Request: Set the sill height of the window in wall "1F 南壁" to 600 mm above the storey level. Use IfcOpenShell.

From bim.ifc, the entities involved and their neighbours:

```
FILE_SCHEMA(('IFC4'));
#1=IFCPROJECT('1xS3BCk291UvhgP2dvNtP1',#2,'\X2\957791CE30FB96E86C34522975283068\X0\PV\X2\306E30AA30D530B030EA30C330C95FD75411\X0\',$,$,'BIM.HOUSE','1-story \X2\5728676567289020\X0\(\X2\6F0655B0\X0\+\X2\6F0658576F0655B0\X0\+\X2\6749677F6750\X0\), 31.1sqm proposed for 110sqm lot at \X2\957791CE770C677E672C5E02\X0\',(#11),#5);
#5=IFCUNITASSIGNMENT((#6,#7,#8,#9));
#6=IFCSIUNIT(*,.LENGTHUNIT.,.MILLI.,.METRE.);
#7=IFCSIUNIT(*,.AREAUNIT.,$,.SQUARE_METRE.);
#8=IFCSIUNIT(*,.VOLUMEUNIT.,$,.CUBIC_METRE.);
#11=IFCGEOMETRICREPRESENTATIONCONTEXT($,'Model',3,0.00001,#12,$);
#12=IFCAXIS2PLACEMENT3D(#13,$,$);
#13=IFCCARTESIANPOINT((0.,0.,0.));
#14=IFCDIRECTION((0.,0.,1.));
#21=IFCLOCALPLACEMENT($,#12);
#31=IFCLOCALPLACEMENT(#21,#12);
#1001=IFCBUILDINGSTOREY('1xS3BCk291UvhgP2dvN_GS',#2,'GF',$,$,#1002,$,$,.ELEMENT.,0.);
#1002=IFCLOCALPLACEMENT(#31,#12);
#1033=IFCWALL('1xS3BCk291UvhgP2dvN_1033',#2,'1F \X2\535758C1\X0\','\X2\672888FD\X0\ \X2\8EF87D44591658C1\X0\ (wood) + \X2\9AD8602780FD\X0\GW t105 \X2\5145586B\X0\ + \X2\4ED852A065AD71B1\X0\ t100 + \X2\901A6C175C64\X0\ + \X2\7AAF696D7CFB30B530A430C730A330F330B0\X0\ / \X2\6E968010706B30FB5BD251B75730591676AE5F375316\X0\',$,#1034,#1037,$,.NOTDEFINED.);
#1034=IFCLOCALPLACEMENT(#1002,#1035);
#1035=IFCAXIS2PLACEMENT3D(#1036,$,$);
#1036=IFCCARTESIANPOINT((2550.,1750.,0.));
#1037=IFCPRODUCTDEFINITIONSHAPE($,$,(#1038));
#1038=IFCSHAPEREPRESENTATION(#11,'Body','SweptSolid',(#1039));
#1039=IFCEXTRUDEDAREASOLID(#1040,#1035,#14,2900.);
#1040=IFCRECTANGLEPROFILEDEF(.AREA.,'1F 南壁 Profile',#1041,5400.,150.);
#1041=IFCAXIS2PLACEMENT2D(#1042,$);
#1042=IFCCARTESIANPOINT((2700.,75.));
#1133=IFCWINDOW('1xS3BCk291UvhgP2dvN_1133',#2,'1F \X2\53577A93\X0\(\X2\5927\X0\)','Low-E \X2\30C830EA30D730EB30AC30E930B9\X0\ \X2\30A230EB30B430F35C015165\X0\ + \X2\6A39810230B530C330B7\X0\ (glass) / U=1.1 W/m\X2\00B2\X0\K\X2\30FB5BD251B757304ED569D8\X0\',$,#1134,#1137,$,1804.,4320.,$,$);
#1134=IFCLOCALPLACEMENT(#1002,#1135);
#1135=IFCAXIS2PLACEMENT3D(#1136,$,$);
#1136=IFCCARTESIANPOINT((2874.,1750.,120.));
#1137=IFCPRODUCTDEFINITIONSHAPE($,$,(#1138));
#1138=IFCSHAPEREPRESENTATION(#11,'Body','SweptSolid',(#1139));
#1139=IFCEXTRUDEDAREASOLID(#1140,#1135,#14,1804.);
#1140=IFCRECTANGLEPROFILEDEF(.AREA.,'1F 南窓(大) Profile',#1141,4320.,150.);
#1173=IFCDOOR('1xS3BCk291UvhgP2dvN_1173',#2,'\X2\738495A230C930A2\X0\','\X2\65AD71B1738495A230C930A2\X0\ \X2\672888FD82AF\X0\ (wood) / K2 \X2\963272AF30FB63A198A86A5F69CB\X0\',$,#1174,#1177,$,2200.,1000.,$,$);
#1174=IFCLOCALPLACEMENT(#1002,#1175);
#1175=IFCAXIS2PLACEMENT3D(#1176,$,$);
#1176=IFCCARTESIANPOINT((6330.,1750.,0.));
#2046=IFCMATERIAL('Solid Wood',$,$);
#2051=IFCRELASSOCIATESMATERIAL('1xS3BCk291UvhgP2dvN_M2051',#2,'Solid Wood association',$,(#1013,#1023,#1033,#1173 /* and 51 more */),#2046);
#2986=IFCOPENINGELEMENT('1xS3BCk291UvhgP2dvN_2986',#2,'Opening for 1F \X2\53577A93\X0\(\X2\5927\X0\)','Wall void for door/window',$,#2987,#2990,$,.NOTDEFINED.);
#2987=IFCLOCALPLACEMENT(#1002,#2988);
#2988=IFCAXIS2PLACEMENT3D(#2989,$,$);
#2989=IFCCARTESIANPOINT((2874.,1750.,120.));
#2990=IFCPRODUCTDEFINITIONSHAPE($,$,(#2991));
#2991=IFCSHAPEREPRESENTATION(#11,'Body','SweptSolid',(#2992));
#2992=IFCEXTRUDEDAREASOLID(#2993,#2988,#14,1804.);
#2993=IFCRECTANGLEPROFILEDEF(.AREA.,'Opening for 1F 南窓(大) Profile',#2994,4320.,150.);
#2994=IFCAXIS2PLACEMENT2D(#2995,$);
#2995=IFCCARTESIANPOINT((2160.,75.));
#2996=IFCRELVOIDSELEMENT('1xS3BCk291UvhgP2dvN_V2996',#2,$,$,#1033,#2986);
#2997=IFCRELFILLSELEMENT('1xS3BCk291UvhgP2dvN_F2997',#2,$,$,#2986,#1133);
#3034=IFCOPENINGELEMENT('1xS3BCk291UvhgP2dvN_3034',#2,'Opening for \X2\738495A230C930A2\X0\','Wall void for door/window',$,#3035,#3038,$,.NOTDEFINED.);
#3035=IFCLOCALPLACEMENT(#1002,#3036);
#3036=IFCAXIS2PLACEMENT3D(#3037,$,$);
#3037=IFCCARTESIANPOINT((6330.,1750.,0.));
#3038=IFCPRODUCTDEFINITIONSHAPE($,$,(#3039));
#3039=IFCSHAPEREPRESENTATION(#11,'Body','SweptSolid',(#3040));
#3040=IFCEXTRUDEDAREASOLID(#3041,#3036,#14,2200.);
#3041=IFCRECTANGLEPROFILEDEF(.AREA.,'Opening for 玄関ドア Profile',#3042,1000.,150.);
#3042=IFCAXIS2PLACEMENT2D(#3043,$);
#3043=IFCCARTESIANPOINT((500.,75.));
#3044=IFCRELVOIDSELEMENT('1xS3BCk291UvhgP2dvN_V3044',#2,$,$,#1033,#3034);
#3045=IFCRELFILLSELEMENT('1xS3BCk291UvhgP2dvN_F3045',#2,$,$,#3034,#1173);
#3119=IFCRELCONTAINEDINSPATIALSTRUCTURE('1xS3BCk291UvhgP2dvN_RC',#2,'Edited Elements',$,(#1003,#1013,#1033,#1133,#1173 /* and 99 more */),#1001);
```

```python
import numpy as np
import ifcopenshell
import ifcopenshell.api.geometry
import ifcopenshell.geom
import ifcopenshell.util.element
import ifcopenshell.util.placement
import ifcopenshell.util.shape
import ifcopenshell.util.unit

model = ifcopenshell.open("bim.ifc")
unit_scale = ifcopenshell.util.unit.calculate_unit_scale(model)

window = model.by_guid("1xS3BCk291UvhgP2dvN_1133")
opening = window.FillsVoids[0].RelatingOpeningElement
storey = ifcopenshell.util.element.get_container(window, ifc_class="IfcBuildingStorey")
level = ifcopenshell.util.placement.get_local_placement(storey.ObjectPlacement)[2, 3]

# The opening's origin need not be at the sill, so measure its lowest point.
shape = ifcopenshell.geom.create_shape(ifcopenshell.geom.settings(), opening)
bottom = ifcopenshell.util.shape.get_shape_bottom_elevation(shape, shape.geometry) / unit_scale
dz = level + 0.6 / unit_scale - bottom

shift = np.array([0.0, 0.0, dz])
# The window is not placed relative to its opening, so move both.
for product in (opening, window):
    matrix = ifcopenshell.util.placement.get_local_placement(product.ObjectPlacement)
    matrix[:3, 3] += shift
    ifcopenshell.api.geometry.edit_object_placement(model, product=product, matrix=matrix, is_si=False)

print(f"moved by {dz * unit_scale:+.3f} m")

model.write("bim-out.ifc")
```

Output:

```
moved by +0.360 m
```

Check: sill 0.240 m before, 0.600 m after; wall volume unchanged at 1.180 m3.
